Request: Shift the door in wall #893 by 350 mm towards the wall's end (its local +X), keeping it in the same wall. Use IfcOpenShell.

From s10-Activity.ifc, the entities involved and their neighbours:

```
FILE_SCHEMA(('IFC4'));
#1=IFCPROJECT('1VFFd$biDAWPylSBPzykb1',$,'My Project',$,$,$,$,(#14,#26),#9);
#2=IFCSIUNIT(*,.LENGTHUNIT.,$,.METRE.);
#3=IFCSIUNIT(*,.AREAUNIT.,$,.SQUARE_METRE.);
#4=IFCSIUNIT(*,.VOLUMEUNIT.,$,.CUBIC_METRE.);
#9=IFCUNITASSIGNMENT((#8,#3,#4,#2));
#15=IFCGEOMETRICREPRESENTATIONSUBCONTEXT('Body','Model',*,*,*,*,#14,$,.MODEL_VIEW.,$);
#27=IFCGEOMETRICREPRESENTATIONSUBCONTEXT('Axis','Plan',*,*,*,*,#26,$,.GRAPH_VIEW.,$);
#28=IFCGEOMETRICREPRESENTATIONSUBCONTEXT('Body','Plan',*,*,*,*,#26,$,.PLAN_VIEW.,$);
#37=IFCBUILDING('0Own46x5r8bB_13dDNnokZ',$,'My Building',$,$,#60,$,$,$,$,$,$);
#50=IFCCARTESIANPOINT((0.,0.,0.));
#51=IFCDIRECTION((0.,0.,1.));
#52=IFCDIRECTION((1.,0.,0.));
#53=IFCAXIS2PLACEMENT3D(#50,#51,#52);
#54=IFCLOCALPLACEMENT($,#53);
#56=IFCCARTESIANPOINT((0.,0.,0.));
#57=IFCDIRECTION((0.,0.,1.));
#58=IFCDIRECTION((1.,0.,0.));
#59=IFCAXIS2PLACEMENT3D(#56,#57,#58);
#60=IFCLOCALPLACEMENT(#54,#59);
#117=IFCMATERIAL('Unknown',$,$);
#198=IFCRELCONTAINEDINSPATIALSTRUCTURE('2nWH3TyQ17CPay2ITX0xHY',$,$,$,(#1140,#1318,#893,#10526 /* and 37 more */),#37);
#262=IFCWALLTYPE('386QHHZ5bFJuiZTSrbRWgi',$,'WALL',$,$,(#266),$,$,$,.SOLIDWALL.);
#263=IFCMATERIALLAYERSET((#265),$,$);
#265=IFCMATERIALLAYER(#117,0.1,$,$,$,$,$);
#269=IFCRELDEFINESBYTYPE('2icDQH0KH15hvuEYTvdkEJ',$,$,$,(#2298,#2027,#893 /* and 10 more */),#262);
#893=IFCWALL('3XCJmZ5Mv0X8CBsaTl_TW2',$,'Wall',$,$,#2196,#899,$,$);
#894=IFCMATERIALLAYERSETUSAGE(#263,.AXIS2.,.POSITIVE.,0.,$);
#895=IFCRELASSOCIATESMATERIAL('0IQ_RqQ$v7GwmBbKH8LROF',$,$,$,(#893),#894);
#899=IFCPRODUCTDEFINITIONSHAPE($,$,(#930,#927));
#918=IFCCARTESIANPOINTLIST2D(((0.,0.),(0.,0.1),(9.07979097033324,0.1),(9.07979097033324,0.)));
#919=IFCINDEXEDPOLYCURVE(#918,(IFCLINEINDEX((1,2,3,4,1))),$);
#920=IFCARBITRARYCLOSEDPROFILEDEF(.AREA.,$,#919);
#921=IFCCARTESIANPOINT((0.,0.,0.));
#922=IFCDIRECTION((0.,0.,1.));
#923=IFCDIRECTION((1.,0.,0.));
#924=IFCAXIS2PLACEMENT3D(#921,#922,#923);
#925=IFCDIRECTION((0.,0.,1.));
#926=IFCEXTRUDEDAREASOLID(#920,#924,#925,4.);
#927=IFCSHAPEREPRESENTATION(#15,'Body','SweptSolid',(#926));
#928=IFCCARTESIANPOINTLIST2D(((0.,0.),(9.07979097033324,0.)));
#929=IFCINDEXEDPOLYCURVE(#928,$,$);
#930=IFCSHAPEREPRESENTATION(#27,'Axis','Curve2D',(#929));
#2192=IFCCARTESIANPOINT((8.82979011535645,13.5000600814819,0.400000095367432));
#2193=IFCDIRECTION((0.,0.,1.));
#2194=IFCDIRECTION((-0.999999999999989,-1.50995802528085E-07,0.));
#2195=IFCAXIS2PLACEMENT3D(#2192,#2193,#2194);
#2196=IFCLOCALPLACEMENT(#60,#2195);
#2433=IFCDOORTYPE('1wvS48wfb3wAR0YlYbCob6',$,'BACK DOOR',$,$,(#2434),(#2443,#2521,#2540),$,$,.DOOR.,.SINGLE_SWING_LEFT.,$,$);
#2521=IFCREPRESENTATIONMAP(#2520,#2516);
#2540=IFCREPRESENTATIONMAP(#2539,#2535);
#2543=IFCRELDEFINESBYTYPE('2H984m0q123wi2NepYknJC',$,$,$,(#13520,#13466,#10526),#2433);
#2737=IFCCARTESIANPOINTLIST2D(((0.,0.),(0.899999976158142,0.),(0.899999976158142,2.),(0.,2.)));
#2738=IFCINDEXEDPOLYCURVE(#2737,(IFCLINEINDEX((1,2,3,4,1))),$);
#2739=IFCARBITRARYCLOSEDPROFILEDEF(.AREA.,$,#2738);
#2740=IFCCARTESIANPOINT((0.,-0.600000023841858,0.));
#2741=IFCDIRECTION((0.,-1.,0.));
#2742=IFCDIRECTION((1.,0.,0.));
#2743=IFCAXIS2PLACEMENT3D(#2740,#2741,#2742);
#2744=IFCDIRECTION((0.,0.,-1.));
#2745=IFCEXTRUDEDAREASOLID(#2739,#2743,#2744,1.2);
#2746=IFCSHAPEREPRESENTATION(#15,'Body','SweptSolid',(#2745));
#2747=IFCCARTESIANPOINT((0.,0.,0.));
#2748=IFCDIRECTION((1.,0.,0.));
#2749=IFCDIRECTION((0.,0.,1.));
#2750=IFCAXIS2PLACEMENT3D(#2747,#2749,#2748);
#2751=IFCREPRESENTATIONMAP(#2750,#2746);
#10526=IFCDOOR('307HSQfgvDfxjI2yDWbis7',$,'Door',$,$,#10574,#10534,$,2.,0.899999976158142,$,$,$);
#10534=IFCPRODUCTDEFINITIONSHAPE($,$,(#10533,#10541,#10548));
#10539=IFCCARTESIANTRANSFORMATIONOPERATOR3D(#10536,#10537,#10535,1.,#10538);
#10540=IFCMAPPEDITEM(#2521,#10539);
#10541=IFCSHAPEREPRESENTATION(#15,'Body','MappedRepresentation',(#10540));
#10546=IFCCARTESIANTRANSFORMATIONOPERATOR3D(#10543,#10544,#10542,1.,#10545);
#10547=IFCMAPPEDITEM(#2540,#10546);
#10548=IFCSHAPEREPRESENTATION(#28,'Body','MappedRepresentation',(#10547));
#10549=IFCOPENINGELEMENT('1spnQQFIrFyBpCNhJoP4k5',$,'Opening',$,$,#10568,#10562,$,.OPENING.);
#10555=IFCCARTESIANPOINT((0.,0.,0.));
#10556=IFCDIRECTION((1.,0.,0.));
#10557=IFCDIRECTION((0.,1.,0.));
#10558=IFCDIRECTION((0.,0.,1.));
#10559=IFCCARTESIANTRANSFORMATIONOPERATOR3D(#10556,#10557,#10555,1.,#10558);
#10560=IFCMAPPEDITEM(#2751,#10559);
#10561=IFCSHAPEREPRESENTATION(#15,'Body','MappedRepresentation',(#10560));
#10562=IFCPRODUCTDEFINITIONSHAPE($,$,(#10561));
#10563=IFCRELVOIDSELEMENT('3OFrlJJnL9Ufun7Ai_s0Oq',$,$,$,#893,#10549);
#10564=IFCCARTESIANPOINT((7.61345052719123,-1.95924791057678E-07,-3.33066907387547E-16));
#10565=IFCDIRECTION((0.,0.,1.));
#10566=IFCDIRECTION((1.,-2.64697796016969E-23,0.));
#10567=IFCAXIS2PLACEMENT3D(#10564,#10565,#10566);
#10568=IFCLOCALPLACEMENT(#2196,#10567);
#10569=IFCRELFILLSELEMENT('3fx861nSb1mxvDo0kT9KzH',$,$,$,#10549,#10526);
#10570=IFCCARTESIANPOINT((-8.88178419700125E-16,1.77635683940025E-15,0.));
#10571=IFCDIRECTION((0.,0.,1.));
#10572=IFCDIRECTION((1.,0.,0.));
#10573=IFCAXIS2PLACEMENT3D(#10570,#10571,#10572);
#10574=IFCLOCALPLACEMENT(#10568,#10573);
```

```python
import ifcopenshell
import ifcopenshell.api.geometry
import ifcopenshell.util.placement

model = ifcopenshell.open("s10-Activity.ifc")

door = model.by_id(10526)
opening = door.FillsVoids[0].RelatingOpeningElement
wall = opening.VoidsElements[0].RelatingBuildingElement

wall_matrix = ifcopenshell.util.placement.get_local_placement(wall.ObjectPlacement)
shift = wall_matrix[:3, 0] * 0.35
before = ifcopenshell.util.placement.get_local_placement(door.ObjectPlacement)[:3, 3].copy()

# The door is placed relative to its opening, so it follows when the opening moves.
matrix = ifcopenshell.util.placement.get_local_placement(opening.ObjectPlacement)
matrix[:3, 3] += shift
ifcopenshell.api.geometry.edit_object_placement(
    model, product=opening, matrix=matrix, is_si=False, should_transform_children=True
)

after = ifcopenshell.util.placement.get_local_placement(door.ObjectPlacement)[:3, 3]
print("door moved by", (after - before).round(3) + 0.0)

model.write("s10-Activity-out.ifc")
```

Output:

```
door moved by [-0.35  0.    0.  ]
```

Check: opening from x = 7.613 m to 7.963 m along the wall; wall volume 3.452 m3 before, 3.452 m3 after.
